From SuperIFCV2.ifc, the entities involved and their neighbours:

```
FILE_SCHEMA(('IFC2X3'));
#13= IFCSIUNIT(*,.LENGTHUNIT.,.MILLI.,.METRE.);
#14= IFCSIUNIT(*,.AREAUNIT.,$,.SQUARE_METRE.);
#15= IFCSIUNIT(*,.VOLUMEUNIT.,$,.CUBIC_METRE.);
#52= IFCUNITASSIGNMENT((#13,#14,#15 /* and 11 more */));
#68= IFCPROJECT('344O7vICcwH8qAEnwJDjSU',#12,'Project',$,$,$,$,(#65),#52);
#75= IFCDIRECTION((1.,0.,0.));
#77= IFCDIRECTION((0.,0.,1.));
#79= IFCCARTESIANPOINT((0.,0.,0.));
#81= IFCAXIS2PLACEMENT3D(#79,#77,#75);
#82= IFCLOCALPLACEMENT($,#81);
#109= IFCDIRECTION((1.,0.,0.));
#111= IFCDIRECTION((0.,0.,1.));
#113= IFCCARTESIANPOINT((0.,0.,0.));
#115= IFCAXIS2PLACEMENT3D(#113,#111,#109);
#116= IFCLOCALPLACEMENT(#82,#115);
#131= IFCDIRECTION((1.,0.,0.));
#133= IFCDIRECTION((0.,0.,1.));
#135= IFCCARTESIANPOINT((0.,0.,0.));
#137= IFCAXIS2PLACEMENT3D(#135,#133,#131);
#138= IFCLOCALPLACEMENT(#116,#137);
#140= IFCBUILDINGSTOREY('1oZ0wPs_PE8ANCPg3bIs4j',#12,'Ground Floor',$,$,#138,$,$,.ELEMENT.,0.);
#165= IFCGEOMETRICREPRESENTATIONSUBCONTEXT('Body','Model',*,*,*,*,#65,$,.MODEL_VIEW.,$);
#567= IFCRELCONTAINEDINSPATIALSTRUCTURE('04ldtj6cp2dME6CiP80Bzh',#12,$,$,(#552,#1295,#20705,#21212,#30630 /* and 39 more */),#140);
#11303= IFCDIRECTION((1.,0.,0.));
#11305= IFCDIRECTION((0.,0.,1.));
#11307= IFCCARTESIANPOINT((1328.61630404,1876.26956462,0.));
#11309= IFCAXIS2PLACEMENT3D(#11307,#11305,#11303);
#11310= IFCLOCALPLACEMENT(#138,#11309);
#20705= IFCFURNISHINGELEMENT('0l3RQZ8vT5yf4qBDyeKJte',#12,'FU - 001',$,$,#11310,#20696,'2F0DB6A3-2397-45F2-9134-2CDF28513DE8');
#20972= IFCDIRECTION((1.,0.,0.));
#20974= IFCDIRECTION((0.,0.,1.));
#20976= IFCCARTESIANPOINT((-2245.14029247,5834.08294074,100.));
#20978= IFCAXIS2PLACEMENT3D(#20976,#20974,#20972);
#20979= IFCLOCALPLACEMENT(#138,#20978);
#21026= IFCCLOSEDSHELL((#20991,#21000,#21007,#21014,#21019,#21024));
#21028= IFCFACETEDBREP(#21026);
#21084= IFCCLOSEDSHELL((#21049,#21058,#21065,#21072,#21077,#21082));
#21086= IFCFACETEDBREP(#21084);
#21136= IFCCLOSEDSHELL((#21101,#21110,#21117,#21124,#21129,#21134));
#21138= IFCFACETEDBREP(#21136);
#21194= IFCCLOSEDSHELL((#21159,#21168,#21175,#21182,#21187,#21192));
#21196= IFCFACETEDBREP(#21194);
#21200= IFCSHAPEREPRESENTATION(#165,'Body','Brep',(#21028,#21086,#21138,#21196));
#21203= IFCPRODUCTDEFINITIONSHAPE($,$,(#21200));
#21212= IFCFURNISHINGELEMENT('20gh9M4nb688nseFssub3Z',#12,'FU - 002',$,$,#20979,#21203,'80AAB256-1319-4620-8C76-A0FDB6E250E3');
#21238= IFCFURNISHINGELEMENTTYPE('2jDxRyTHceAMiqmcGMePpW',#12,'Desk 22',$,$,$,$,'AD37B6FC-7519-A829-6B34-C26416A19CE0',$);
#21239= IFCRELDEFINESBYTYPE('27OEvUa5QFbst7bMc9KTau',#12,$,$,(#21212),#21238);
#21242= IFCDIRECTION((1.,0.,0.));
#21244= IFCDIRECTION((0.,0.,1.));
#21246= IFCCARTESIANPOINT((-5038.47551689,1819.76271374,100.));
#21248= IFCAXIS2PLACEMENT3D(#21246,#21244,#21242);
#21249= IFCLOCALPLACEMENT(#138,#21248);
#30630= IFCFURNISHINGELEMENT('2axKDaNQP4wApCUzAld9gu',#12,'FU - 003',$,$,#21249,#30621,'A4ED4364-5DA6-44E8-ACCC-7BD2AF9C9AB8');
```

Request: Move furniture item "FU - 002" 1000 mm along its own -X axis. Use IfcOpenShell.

```python
import ifcopenshell
import ifcopenshell.api.geometry
import ifcopenshell.util.placement

model = ifcopenshell.open("SuperIFCV2.ifc")

item = model.by_guid("20gh9M4nb688nseFssub3Z")
matrix = ifcopenshell.util.placement.get_local_placement(item.ObjectPlacement)
matrix[:3, 3] -= matrix[:3, 0] * 1000.0
ifcopenshell.api.geometry.edit_object_placement(model, product=item, matrix=matrix, is_si=False)

print(ifcopenshell.util.placement.get_local_placement(item.ObjectPlacement).round(3) + 0.0)

model.write("SuperIFCV2_rev.ifc")
```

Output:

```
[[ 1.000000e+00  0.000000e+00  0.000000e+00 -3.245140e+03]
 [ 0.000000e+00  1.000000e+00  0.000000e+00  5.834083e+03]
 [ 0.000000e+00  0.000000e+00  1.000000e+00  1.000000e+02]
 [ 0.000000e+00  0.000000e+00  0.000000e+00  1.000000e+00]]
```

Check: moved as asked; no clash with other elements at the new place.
